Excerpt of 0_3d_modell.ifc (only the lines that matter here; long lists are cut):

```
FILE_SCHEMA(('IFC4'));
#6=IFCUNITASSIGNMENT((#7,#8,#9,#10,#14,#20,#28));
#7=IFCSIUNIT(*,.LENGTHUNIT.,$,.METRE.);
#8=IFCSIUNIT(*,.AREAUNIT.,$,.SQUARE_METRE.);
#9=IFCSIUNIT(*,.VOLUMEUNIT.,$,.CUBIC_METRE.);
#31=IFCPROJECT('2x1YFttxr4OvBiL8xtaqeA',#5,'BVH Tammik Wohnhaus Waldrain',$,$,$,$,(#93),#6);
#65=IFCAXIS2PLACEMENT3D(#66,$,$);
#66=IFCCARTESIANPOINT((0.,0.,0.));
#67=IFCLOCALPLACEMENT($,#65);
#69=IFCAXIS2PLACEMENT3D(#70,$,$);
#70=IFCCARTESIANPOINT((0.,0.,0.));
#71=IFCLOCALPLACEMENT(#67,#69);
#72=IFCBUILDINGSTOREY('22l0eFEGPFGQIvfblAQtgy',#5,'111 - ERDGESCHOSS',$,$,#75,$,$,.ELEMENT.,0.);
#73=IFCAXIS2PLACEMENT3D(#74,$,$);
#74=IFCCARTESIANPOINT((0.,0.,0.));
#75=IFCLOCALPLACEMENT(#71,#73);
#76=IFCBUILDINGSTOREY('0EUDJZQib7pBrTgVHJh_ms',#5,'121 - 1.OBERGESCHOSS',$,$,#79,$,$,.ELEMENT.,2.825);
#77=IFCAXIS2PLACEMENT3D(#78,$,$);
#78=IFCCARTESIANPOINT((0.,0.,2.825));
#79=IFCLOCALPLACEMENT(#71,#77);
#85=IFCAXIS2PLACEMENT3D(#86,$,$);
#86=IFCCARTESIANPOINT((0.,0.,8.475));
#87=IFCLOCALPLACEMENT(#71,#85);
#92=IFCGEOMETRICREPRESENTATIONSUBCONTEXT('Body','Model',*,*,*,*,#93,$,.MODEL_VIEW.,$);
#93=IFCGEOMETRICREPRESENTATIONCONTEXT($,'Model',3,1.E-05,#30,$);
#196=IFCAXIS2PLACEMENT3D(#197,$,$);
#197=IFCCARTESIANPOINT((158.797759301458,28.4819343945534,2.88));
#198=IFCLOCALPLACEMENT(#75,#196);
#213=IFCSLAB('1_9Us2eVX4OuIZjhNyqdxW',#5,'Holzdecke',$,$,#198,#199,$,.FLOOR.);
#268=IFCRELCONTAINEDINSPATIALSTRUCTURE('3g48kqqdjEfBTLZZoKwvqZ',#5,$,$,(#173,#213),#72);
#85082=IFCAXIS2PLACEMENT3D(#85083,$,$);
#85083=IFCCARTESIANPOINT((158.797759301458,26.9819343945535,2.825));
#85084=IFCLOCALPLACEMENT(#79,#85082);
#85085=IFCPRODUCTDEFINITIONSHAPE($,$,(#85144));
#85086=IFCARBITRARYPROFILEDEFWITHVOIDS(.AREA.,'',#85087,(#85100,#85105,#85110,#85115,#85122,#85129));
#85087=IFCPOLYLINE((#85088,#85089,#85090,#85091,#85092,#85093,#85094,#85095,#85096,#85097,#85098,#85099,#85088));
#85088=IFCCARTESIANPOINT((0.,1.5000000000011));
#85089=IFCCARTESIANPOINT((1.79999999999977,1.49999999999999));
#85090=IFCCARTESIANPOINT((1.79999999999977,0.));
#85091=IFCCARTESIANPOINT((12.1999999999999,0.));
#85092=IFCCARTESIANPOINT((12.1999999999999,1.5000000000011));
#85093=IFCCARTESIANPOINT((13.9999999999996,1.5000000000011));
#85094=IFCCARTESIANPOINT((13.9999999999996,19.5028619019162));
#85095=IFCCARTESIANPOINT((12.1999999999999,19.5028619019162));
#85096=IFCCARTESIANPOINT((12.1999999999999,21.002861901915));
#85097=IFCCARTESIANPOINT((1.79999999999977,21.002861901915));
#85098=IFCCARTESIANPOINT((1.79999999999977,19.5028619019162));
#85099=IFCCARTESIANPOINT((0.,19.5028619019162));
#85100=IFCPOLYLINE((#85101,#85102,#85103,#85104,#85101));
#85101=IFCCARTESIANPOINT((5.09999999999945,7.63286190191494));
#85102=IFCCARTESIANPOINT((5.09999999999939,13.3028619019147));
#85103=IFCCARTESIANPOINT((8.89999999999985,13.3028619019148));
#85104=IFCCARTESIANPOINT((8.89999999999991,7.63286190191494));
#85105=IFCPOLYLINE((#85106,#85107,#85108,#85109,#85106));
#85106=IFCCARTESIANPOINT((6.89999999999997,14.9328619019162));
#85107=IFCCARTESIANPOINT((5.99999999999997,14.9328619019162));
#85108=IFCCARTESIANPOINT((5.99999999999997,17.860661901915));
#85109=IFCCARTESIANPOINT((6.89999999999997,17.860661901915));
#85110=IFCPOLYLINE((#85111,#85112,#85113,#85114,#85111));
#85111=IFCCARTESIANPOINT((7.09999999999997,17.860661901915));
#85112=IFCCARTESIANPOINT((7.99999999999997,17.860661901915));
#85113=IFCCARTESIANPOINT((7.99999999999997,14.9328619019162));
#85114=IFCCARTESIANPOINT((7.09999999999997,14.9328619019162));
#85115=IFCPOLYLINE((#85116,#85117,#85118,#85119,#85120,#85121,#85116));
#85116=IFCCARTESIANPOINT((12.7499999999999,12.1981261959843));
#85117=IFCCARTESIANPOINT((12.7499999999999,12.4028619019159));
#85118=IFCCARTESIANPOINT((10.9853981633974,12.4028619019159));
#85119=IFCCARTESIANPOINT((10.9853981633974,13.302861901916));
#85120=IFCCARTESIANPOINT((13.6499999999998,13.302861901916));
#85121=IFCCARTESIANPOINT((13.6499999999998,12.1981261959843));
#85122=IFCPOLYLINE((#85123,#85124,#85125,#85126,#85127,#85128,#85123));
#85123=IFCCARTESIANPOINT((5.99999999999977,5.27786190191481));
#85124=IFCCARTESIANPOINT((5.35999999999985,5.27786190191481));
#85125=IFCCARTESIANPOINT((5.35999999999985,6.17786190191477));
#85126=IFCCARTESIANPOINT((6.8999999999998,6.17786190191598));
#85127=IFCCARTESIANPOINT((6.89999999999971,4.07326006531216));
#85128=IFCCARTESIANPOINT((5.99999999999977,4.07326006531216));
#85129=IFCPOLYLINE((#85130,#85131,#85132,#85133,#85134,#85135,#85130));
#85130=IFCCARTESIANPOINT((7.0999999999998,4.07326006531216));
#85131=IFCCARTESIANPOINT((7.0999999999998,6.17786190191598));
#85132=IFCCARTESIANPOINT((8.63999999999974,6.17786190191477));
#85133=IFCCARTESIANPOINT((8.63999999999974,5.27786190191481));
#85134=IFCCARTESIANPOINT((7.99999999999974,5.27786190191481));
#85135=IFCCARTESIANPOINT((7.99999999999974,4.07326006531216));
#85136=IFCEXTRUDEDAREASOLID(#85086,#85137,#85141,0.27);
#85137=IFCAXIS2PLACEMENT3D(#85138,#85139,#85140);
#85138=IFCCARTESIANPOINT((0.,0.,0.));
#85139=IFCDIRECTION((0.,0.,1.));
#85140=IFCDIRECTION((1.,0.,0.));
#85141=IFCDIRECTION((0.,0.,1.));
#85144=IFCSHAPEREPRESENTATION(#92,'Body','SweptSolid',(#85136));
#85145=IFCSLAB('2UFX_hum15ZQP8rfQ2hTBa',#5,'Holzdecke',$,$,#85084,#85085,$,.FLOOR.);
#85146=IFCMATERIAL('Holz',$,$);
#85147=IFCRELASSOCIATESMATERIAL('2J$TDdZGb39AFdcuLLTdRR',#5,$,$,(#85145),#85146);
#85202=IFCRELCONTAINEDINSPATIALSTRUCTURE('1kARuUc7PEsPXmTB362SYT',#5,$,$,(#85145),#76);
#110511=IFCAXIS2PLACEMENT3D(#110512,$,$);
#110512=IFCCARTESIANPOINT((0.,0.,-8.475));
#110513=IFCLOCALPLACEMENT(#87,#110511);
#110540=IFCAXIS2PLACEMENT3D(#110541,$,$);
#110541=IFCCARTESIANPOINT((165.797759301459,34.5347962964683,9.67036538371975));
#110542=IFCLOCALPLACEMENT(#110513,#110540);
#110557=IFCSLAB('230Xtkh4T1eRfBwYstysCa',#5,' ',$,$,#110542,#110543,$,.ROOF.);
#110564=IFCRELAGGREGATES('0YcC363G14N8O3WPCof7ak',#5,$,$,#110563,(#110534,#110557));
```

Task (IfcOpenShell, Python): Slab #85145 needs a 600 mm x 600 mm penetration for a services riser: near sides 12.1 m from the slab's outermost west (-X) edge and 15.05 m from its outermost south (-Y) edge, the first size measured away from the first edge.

```python
import numpy as np
import ifcopenshell
import ifcopenshell.api.feature
import ifcopenshell.api.geometry
import ifcopenshell.api.root
import ifcopenshell.geom
import ifcopenshell.util.placement
import ifcopenshell.util.representation
import ifcopenshell.util.shape
import ifcopenshell.util.unit

model = ifcopenshell.open("0_3d_modell.ifc")
unit_scale = ifcopenshell.util.unit.calculate_unit_scale(model)
settings = ifcopenshell.geom.settings()


def volume(element):
    """Net volume in cubic metres, openings subtracted."""
    shape = ifcopenshell.geom.create_shape(settings, element)
    return ifcopenshell.util.shape.get_volume(shape.geometry)


slab = model.by_guid("2UFX_hum15ZQP8rfQ2hTBa")
before = volume(slab)

# Extent in the slab's own axes, in metres. The edges named are its -X and -Y sides.
slab_shape = ifcopenshell.geom.create_shape(settings, slab)
vertices = ifcopenshell.util.shape.get_vertices(slab_shape.geometry)
x_min, y_min, bottom = vertices.min(axis=0)
top = vertices[:, 2].max()

opening = ifcopenshell.api.root.create_entity(model, ifc_class="IfcOpeningElement", name="Services riser opening", predefined_type="OPENING")
context = ifcopenshell.util.representation.get_context(model, "Model", "Body", "MODEL_VIEW")
width, depth = 0.6, 0.6
outline = [(0.0, 0.0), (width, 0.0), (width, depth), (0.0, depth), (0.0, 0.0)]
# Overshoot both faces by 50 mm so the cut is clean.
shape = ifcopenshell.api.geometry.add_slab_representation(
    model, context=context, depth=top - bottom + 0.1, polyline=outline
)
ifcopenshell.api.geometry.assign_representation(model, product=opening, representation=shape)

matrix = ifcopenshell.util.placement.get_local_placement(slab.ObjectPlacement)
matrix[:, 3] = matrix @ np.append(np.array([x_min + 12.1, y_min + 15.05, bottom - 0.05]) / unit_scale, 1.0)
ifcopenshell.api.geometry.edit_object_placement(model, product=opening, matrix=matrix, is_si=False)
ifcopenshell.api.feature.add_feature(model, feature=opening, element=slab)

after = volume(slab)

print(f"slab volume {before:.3f} -> {after:.3f} m3")

model.write("0_3d_modell_rev.ifc")
```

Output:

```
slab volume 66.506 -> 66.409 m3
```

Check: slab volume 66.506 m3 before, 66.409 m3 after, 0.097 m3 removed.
